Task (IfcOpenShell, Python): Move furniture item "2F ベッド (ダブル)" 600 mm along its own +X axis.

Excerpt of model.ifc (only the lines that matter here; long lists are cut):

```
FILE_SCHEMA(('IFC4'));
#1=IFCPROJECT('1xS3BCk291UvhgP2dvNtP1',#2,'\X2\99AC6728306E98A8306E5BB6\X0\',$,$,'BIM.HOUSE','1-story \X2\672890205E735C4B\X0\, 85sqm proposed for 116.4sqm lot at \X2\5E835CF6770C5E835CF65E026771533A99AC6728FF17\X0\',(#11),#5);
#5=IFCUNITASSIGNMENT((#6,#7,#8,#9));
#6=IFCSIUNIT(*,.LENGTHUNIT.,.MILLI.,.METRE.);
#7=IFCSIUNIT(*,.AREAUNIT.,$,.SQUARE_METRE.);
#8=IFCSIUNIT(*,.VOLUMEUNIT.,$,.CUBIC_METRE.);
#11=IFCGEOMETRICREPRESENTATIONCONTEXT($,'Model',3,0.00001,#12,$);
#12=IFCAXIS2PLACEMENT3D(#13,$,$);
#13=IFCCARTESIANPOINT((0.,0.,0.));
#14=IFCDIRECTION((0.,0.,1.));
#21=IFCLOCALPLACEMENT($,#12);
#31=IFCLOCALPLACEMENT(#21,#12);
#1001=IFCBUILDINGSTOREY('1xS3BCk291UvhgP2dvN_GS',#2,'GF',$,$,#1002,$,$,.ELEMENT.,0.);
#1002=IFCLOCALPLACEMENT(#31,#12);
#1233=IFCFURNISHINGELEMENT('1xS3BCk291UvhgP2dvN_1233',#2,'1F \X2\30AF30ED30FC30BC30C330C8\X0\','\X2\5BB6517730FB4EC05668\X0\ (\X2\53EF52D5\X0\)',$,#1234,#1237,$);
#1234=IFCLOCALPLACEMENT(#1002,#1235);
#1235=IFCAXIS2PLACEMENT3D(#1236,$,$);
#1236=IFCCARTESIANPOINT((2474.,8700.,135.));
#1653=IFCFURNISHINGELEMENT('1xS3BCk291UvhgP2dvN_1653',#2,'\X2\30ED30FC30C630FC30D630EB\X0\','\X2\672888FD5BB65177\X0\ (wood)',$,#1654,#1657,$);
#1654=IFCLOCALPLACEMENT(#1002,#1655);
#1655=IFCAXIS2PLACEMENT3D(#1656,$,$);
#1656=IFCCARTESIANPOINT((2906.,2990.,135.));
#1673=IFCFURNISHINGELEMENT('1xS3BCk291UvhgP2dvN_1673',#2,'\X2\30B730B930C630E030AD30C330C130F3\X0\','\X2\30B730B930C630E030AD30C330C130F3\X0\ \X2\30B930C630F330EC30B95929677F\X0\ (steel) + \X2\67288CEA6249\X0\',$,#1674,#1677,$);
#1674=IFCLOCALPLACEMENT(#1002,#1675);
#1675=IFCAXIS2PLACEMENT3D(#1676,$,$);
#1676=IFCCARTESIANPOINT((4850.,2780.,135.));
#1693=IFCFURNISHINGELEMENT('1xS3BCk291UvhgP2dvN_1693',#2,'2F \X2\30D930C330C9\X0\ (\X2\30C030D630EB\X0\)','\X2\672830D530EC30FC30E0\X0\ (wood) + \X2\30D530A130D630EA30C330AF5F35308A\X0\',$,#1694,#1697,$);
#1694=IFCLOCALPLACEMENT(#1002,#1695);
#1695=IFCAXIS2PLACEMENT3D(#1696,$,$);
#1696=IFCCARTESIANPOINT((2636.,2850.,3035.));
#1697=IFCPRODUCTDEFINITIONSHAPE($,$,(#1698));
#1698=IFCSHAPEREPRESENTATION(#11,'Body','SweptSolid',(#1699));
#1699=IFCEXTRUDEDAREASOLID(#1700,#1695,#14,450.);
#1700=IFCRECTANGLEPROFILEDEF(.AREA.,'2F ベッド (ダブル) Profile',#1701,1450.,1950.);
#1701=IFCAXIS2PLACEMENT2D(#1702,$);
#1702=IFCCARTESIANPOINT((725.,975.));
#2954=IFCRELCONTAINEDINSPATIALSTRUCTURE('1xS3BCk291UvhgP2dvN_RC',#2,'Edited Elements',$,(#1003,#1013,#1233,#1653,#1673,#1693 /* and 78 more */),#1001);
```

```python
import ifcopenshell
import ifcopenshell.api.geometry
import ifcopenshell.util.placement
import ifcopenshell.util.unit

model = ifcopenshell.open("model.ifc")
unit_scale = ifcopenshell.util.unit.calculate_unit_scale(model)

item = model.by_guid("1xS3BCk291UvhgP2dvN_1693")
matrix = ifcopenshell.util.placement.get_local_placement(item.ObjectPlacement)
matrix[:3, 3] += matrix[:3, 0] * 0.6 / unit_scale
ifcopenshell.api.geometry.edit_object_placement(model, product=item, matrix=matrix, is_si=False)

print(ifcopenshell.util.placement.get_local_placement(item.ObjectPlacement).round(3) + 0.0)

model.write("model_v2.ifc")
```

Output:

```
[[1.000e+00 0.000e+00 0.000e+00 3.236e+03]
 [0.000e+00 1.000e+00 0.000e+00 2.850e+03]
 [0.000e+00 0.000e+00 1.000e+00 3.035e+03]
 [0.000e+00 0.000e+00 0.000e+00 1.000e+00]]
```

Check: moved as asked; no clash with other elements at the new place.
